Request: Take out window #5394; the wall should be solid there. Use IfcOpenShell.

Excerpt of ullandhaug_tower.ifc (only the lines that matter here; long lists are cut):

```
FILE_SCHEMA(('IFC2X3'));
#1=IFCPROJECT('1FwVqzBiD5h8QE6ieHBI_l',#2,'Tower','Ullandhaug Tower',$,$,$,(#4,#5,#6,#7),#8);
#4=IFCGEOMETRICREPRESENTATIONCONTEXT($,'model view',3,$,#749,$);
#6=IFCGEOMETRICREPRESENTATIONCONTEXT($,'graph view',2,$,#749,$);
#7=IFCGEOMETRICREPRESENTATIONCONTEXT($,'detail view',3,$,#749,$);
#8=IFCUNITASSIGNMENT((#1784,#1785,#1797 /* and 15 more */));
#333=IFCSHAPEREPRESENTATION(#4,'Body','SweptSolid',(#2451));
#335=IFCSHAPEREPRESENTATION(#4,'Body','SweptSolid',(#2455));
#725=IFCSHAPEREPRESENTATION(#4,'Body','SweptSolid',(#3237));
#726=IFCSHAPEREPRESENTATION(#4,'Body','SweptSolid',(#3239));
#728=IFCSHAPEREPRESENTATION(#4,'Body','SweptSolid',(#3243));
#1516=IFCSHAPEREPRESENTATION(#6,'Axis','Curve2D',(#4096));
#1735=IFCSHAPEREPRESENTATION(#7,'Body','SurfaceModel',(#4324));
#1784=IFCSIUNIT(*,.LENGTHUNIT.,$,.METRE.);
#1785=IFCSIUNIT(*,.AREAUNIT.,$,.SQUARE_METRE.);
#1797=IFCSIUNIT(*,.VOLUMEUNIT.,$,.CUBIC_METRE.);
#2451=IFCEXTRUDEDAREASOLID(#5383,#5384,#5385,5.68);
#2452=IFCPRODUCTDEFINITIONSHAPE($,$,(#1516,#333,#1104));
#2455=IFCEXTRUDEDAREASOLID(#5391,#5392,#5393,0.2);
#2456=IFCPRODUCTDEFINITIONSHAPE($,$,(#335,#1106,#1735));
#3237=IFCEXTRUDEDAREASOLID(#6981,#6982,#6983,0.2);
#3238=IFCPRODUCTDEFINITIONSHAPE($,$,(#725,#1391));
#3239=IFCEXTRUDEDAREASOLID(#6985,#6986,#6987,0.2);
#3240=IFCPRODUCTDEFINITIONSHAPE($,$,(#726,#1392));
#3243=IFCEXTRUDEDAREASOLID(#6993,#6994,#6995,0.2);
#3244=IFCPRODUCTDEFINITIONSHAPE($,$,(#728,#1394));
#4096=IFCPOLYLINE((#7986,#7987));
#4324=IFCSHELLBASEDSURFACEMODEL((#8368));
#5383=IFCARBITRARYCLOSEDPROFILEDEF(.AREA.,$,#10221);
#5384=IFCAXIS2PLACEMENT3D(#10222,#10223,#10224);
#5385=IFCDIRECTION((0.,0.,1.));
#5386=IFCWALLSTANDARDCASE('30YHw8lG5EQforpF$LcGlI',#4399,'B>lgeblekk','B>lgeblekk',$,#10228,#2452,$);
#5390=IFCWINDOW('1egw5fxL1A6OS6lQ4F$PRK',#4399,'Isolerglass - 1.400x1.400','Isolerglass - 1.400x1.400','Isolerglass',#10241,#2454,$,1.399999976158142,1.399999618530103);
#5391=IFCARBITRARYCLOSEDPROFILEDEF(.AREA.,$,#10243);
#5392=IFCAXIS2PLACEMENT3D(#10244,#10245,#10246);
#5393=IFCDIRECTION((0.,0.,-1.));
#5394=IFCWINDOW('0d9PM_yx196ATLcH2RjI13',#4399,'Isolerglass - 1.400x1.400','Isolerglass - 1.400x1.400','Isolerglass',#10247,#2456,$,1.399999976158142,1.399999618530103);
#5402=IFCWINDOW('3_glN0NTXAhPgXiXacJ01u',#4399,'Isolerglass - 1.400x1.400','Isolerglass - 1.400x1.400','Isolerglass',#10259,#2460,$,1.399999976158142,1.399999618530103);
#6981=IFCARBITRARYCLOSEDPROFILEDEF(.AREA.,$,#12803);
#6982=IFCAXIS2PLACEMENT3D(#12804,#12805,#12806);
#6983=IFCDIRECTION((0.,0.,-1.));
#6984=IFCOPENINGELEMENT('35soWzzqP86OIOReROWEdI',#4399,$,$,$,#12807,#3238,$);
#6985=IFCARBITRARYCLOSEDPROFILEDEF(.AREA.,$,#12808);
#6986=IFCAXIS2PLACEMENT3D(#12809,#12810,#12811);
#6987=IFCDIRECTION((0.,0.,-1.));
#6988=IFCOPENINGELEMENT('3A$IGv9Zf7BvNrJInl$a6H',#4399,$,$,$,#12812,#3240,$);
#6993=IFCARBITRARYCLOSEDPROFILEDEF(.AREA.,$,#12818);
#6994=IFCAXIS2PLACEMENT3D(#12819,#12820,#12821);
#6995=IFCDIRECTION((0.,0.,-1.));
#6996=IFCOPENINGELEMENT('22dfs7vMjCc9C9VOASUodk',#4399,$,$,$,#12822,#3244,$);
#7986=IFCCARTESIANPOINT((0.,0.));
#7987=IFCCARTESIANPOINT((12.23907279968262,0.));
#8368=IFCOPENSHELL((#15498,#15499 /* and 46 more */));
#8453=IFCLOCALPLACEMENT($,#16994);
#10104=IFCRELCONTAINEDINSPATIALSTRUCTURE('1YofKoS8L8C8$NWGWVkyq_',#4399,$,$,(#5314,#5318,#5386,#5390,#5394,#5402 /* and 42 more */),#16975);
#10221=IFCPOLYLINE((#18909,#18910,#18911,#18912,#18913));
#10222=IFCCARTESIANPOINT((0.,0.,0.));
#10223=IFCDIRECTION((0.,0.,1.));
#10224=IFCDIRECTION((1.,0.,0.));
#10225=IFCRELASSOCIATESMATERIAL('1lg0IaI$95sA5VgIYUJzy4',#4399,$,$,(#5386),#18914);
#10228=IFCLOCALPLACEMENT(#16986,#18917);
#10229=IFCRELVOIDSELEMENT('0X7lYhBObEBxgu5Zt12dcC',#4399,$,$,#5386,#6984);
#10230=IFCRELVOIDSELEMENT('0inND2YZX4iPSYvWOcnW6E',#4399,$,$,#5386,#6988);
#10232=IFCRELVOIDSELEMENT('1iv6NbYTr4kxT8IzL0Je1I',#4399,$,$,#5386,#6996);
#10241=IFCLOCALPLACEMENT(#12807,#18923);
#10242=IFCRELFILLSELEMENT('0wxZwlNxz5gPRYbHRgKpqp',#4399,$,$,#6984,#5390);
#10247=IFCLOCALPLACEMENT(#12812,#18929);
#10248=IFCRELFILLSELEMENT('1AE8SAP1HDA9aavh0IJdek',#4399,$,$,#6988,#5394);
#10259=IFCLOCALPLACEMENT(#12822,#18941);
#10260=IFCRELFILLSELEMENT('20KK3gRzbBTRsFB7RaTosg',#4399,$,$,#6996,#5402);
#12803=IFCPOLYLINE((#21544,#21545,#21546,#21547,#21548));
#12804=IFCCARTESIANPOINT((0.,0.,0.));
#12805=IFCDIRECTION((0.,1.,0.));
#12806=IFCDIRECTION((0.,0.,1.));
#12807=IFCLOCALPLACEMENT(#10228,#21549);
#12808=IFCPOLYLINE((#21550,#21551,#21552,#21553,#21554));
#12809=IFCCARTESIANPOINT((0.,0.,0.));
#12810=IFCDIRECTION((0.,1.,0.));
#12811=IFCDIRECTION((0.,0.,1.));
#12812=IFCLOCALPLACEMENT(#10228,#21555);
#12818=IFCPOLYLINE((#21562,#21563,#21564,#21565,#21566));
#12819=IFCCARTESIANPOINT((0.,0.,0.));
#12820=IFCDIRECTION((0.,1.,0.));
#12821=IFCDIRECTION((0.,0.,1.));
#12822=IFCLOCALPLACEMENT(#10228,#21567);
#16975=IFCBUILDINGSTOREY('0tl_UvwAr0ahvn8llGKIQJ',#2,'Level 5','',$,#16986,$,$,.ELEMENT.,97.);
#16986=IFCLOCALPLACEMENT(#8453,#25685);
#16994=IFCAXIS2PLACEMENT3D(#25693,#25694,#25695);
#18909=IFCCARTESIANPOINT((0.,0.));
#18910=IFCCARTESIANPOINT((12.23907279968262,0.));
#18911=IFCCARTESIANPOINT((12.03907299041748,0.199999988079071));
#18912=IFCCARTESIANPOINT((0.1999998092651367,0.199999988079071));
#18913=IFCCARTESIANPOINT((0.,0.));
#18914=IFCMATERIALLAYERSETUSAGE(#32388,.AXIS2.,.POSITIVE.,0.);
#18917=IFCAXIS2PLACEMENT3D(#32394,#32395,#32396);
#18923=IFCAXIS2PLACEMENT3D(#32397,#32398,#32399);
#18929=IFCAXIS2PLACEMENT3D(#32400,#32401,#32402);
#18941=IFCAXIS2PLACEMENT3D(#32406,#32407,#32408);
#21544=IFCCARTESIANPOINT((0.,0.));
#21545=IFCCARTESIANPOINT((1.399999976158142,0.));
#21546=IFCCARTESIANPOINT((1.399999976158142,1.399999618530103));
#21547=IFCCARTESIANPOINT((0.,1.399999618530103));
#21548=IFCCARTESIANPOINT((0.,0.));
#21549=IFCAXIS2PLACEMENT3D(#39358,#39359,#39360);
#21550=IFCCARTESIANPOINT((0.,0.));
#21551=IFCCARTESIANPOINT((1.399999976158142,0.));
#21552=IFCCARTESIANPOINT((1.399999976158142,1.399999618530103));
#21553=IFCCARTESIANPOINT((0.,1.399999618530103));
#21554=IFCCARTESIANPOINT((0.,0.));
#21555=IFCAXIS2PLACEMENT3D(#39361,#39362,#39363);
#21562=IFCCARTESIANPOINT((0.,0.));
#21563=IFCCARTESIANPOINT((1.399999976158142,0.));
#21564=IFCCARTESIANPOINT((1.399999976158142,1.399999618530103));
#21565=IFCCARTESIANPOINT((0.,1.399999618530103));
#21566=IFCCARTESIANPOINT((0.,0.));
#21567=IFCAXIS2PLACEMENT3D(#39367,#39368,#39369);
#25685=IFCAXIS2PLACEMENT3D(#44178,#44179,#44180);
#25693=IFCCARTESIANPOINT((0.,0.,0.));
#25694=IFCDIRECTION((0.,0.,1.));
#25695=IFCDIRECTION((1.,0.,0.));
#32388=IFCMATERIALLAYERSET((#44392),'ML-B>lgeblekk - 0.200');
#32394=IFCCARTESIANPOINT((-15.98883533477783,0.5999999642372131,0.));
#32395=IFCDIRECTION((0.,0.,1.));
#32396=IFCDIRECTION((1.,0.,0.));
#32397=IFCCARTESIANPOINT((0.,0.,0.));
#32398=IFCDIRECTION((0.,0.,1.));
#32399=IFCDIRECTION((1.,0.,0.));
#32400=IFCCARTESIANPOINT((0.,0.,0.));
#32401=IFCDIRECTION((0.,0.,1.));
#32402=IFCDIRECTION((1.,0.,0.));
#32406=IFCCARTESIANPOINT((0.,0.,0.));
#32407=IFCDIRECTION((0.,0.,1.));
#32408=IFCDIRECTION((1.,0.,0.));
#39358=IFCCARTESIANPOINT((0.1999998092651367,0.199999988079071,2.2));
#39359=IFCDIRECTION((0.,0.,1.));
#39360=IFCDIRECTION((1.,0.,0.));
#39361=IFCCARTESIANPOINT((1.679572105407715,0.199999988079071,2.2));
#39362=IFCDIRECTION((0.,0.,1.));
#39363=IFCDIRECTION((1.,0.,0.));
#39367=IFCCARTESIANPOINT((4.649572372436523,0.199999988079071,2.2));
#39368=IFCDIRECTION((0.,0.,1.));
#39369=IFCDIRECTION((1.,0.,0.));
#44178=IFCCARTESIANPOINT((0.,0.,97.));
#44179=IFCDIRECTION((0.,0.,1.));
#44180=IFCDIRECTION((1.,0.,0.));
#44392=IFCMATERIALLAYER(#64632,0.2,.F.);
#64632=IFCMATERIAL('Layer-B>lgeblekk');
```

```python
import ifcopenshell
import ifcopenshell.api.feature
import ifcopenshell.api.root
import ifcopenshell.geom
import ifcopenshell.util.shape

model = ifcopenshell.open("ullandhaug_tower.ifc")
settings = ifcopenshell.geom.settings()


def volume(element):
    """Net volume in cubic metres, openings subtracted."""
    shape = ifcopenshell.geom.create_shape(settings, element)
    return ifcopenshell.util.shape.get_volume(shape.geometry)


window = model.by_guid("0d9PM_yx196ATLcH2RjI13")
opening = window.FillsVoids[0].RelatingOpeningElement
wall = opening.VoidsElements[0].RelatingBuildingElement
before = volume(wall)

ifcopenshell.api.root.remove_product(model, product=window)
ifcopenshell.api.feature.remove_feature(model, feature=opening)

after = volume(wall)

print(f"wall volume {before:.3f} -> {after:.3f} m3")

model.write("ullandhaug_tower_edited.ifc")
```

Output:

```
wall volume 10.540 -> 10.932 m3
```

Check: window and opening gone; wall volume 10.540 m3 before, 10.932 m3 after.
